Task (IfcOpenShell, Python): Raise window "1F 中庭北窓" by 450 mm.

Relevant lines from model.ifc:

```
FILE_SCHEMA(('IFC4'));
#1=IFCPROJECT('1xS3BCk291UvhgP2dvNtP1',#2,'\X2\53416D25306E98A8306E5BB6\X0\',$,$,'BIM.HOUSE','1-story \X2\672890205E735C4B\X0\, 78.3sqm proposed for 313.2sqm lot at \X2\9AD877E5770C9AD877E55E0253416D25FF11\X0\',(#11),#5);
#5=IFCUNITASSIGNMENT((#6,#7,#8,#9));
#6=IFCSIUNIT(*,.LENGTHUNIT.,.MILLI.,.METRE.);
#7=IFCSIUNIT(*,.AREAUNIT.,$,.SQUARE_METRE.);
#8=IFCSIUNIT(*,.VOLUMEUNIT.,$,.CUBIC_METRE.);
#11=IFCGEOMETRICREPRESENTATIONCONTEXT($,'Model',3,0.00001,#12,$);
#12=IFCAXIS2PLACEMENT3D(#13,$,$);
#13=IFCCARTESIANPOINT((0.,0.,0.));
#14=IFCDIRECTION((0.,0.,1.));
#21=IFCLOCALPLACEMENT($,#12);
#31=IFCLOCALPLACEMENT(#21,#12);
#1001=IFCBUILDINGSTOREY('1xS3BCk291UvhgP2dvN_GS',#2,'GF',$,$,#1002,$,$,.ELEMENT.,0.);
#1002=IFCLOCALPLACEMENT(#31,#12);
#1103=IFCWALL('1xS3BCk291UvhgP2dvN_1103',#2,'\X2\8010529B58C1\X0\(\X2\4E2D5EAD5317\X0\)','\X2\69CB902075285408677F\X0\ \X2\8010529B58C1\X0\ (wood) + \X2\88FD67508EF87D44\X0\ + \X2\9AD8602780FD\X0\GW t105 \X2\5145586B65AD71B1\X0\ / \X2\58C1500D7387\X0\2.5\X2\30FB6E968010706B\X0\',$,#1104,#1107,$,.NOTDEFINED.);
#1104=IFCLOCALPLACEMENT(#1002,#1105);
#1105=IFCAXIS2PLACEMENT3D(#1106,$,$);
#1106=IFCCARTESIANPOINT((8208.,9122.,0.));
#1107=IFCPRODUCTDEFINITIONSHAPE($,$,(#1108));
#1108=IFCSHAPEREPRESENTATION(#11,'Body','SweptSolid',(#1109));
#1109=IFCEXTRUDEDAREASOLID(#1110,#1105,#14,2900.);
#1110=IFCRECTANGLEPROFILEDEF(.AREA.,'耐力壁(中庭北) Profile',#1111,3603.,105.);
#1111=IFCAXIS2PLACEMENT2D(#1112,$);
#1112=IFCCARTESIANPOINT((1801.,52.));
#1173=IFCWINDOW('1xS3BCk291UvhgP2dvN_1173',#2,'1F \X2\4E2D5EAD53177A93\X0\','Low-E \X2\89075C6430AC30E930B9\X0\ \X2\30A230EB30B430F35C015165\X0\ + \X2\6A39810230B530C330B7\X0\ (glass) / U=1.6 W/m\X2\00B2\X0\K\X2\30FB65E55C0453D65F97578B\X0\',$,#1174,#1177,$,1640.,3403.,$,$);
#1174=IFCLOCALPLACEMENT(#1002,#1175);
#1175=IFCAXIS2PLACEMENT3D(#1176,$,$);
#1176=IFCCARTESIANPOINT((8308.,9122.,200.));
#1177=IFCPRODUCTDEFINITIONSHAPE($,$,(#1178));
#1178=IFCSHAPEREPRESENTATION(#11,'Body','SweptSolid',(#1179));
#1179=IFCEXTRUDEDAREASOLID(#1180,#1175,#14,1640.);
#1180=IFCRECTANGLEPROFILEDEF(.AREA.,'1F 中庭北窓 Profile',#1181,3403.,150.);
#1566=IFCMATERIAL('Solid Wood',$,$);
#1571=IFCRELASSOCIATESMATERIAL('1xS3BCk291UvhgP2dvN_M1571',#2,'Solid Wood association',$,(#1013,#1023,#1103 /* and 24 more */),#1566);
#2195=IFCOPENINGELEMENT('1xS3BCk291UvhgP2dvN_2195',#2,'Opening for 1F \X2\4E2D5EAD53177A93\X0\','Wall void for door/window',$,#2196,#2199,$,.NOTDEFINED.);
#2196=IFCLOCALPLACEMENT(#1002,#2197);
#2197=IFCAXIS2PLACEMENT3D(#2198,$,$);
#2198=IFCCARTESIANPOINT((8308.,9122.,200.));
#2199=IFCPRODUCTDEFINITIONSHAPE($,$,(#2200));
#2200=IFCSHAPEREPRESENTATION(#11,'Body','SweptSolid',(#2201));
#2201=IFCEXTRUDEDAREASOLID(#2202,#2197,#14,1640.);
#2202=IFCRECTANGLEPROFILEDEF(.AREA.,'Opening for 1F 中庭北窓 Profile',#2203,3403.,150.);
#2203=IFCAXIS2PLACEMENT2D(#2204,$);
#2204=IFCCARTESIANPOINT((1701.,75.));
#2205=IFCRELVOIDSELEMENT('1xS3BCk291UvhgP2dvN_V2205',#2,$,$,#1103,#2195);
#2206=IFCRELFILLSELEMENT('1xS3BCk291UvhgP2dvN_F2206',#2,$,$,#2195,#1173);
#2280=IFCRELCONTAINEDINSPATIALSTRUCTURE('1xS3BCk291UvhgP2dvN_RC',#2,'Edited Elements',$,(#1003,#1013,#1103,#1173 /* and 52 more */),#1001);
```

```python
import numpy as np
import ifcopenshell
import ifcopenshell.api.geometry
import ifcopenshell.util.placement
import ifcopenshell.util.unit

model = ifcopenshell.open("model.ifc")
unit_scale = ifcopenshell.util.unit.calculate_unit_scale(model)

window = model.by_guid("1xS3BCk291UvhgP2dvN_1173")
opening = window.FillsVoids[0].RelatingOpeningElement
dz = 0.45 / unit_scale

shift = np.array([0.0, 0.0, dz])
# The window is not placed relative to its opening, so move both.
for product in (opening, window):
    matrix = ifcopenshell.util.placement.get_local_placement(product.ObjectPlacement)
    matrix[:3, 3] += shift
    ifcopenshell.api.geometry.edit_object_placement(model, product=product, matrix=matrix, is_si=False)

print(f"moved by {dz * unit_scale:+.3f} m")

model.write("model_v2.ifc")
```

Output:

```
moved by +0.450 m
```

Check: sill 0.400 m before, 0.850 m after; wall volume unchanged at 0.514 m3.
